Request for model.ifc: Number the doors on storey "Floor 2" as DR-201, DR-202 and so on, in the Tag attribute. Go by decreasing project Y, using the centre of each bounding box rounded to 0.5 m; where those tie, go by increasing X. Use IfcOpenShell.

First a look at what the model holds.

```python
import ifcopenshell
import ifcopenshell.util.element
import ifcopenshell.util.placement

model = ifcopenshell.open("model.ifc")
print(model.schema)
storey = next(s for s in model.by_type("IfcBuildingStorey") if s.Name == "Floor 2")
doors = [e for e in ifcopenshell.util.element.get_decomposition(storey) if e.is_a("IfcDoor")]
for e in sorted(doors, key=lambda e: e.id()):
    origin = ifcopenshell.util.placement.get_local_placement(e.ObjectPlacement)[:3, 3]
    print(e.id(), e.Tag, e.Name, origin.round(2) + 0.0, sep=" | ")
```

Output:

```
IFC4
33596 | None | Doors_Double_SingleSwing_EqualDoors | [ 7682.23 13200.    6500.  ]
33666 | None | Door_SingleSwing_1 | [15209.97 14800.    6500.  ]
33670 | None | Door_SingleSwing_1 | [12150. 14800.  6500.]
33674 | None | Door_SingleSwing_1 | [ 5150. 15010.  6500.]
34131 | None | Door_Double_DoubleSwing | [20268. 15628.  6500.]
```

```python
import ifcopenshell
import ifcopenshell.geom
import ifcopenshell.util.element
import ifcopenshell.util.shape

model = ifcopenshell.open("model.ifc")
settings = ifcopenshell.geom.settings()
settings.set("use-world-coords", True)


def centre(element):
    shape = ifcopenshell.geom.create_shape(settings, element)
    return ifcopenshell.util.shape.get_bbox_centroid(shape.geometry)


storey = next(s for s in model.by_type("IfcBuildingStorey") if s.Name == "Floor 2")
doors = [e for e in ifcopenshell.util.element.get_decomposition(storey) if e.is_a("IfcDoor")]

# Insertion points can sit at a corner or the storey origin, so sort by the geometry (in metres).
centres = {e: centre(e) for e in doors}
doors.sort(key=lambda e: (-round(centres[e][1] / 0.5), centres[e][0]))

for i, e in enumerate(doors, start=1):
    number = f"DR-2{i:02d}"
    e.Tag = number
    print(e.id(), number)

model.write("model_edited.ifc")
```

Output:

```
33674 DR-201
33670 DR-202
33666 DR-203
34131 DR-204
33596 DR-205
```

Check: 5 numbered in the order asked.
